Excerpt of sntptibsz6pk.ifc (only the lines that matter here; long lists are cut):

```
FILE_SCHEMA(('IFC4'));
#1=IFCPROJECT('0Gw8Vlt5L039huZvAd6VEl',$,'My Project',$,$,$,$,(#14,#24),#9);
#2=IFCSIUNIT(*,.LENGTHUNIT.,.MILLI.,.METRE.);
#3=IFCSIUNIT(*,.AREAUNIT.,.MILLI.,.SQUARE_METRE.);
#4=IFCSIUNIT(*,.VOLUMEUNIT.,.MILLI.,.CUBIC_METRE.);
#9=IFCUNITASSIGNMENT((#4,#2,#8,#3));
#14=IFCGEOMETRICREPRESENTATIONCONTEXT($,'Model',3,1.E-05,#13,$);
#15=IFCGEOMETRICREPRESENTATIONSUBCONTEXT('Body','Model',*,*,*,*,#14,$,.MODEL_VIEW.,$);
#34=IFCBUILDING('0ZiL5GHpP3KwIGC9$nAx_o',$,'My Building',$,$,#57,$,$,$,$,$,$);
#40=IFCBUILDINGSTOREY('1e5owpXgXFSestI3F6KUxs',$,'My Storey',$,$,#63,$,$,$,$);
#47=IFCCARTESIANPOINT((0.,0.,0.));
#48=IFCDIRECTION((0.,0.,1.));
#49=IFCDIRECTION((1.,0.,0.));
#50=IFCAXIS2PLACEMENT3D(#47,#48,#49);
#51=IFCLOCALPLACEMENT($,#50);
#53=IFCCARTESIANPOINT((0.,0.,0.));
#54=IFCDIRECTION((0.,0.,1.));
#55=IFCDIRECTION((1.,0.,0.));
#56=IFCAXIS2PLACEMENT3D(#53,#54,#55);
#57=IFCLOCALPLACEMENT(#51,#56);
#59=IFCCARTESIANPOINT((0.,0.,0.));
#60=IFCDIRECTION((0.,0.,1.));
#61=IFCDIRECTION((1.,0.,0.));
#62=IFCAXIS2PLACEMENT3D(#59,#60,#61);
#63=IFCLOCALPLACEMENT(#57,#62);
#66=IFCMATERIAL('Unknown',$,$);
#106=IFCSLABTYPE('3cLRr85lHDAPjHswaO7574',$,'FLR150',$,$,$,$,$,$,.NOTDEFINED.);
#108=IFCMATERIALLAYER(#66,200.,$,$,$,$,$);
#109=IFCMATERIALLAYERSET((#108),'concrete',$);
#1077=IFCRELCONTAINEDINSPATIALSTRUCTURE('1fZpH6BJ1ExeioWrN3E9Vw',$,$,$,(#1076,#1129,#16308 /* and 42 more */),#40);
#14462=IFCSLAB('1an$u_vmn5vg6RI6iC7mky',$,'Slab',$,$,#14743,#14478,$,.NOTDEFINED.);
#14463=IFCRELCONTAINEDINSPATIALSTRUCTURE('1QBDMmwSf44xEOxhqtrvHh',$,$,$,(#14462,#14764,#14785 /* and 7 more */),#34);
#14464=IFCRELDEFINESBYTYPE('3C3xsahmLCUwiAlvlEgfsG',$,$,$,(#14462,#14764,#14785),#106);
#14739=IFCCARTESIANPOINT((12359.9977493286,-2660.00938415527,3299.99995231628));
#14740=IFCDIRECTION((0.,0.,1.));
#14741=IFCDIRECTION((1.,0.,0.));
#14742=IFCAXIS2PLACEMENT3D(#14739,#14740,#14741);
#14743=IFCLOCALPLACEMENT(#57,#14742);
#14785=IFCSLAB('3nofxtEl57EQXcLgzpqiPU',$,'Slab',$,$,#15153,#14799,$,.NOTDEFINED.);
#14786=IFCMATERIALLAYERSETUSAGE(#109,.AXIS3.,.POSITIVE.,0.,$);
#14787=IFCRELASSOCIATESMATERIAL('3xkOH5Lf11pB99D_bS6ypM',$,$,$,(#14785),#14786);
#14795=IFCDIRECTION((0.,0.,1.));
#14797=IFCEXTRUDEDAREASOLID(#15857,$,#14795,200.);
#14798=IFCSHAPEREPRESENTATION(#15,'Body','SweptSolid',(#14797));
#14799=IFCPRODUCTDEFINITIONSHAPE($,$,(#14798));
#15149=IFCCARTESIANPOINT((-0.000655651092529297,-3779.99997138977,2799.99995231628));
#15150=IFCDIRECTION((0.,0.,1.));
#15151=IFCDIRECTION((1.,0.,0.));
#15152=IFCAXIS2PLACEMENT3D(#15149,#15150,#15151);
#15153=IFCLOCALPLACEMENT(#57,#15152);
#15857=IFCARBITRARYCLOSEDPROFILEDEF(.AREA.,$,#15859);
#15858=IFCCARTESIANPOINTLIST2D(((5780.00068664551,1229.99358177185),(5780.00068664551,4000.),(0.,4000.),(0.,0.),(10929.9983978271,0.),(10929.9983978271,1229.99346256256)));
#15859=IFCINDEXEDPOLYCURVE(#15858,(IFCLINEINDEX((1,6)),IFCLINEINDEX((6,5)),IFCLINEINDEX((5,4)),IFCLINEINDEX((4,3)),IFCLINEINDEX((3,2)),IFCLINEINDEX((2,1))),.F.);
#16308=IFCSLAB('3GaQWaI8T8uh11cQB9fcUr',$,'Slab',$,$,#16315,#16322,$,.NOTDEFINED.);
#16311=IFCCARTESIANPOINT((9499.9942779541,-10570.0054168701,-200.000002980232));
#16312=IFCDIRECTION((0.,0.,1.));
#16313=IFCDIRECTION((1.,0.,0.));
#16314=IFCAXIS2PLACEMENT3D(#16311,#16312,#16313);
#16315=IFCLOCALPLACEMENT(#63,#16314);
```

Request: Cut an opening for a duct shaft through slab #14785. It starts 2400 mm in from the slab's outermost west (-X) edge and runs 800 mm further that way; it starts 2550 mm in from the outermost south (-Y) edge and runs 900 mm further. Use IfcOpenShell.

```python
import numpy as np
import ifcopenshell
import ifcopenshell.api.feature
import ifcopenshell.api.geometry
import ifcopenshell.api.root
import ifcopenshell.geom
import ifcopenshell.util.placement
import ifcopenshell.util.representation
import ifcopenshell.util.shape
import ifcopenshell.util.unit

model = ifcopenshell.open("sntptibsz6pk.ifc")
unit_scale = ifcopenshell.util.unit.calculate_unit_scale(model)
settings = ifcopenshell.geom.settings()


def volume(element):
    """Net volume in cubic metres, openings subtracted."""
    shape = ifcopenshell.geom.create_shape(settings, element)
    return ifcopenshell.util.shape.get_volume(shape.geometry)


slab = model.by_guid("3nofxtEl57EQXcLgzpqiPU")
before = volume(slab)

# Extent in the slab's own axes, in metres. The edges named are its -X and -Y sides.
slab_shape = ifcopenshell.geom.create_shape(settings, slab)
vertices = ifcopenshell.util.shape.get_vertices(slab_shape.geometry)
x_min, y_min, bottom = vertices.min(axis=0)
top = vertices[:, 2].max()

opening = ifcopenshell.api.root.create_entity(model, ifc_class="IfcOpeningElement", name="Duct shaft opening", predefined_type="OPENING")
context = ifcopenshell.util.representation.get_context(model, "Model", "Body", "MODEL_VIEW")
width, depth = 0.8, 0.9
outline = [(0.0, 0.0), (width, 0.0), (width, depth), (0.0, depth), (0.0, 0.0)]
# Overshoot both faces by 50 mm so the cut is clean.
shape = ifcopenshell.api.geometry.add_slab_representation(
    model, context=context, depth=top - bottom + 0.1, polyline=outline
)
ifcopenshell.api.geometry.assign_representation(model, product=opening, representation=shape)

matrix = ifcopenshell.util.placement.get_local_placement(slab.ObjectPlacement)
matrix[:, 3] = matrix @ np.append(np.array([x_min + 2.4, y_min + 2.55, bottom - 0.05]) / unit_scale, 1.0)
ifcopenshell.api.geometry.edit_object_placement(model, product=opening, matrix=matrix, is_si=False)
ifcopenshell.api.feature.add_feature(model, feature=opening, element=slab)

after = volume(slab)

print(f"slab volume {before:.3f} -> {after:.3f} m3")

model.write("sntptibsz6pk_edited.ifc")
```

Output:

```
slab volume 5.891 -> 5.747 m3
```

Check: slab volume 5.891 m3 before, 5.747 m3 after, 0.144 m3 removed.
